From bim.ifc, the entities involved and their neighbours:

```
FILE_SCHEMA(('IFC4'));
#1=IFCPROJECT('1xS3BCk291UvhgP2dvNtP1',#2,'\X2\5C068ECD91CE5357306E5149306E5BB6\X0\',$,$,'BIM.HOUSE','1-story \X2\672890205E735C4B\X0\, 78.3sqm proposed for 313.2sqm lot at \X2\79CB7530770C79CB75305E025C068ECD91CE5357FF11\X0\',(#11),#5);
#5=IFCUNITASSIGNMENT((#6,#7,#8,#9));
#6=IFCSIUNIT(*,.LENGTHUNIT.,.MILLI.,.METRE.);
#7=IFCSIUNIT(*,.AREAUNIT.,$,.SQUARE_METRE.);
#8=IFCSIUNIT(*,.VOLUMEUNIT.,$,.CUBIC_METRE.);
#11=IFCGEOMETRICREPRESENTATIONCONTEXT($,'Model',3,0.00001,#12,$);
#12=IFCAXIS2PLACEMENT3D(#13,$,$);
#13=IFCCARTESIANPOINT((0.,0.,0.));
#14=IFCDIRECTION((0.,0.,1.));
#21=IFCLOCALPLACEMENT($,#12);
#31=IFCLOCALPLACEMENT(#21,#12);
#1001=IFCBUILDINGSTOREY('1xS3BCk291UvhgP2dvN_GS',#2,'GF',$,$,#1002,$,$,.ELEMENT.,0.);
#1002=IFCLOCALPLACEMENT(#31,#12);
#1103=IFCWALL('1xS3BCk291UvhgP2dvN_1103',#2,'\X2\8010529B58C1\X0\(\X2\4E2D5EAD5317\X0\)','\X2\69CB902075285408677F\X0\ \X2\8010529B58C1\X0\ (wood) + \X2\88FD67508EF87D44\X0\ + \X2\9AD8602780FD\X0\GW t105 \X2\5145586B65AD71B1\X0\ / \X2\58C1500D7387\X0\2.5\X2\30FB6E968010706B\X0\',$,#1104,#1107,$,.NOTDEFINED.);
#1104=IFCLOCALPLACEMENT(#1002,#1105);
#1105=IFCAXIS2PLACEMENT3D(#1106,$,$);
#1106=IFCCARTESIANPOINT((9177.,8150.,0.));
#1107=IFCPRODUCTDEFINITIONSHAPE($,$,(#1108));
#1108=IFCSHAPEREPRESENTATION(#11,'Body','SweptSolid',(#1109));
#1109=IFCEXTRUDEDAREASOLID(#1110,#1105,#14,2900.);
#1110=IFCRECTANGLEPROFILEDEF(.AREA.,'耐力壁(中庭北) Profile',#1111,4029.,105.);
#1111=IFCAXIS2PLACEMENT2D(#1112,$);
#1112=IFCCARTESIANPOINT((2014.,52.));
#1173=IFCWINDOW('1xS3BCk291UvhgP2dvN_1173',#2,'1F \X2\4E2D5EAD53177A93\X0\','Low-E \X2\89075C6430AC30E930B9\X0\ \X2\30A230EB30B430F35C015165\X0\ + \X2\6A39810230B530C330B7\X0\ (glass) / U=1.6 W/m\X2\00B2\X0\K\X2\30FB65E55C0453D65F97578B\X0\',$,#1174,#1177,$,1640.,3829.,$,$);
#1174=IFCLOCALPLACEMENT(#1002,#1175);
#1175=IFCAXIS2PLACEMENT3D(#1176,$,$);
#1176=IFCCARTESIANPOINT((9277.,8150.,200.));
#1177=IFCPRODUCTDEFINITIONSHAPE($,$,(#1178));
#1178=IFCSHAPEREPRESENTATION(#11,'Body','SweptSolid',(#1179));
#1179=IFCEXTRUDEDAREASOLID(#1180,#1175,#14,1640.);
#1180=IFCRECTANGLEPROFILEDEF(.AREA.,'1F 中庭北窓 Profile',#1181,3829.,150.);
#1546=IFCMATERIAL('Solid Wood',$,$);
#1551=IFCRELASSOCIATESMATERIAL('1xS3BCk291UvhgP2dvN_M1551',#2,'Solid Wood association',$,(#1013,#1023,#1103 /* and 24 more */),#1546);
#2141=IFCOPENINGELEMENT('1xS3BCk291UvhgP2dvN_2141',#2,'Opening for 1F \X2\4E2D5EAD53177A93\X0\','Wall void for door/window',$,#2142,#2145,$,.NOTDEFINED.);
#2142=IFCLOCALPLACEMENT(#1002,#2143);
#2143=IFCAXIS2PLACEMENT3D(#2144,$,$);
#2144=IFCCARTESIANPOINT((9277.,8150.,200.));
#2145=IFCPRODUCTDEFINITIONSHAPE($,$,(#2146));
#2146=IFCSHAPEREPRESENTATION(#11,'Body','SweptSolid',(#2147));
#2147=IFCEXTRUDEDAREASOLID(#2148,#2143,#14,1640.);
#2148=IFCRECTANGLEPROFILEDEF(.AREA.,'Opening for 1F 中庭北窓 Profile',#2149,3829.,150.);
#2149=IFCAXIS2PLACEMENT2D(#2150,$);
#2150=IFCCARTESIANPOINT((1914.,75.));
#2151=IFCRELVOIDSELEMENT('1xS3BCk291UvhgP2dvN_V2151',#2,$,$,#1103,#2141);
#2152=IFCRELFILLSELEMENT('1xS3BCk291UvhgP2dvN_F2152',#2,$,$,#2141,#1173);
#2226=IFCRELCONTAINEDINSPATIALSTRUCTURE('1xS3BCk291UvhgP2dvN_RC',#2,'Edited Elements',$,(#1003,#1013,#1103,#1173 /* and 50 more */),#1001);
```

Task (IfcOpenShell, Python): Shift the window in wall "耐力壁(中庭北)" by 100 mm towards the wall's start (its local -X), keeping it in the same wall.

```python
import ifcopenshell
import ifcopenshell.api.geometry
import ifcopenshell.util.placement
import ifcopenshell.util.unit

model = ifcopenshell.open("bim.ifc")
unit_scale = ifcopenshell.util.unit.calculate_unit_scale(model)

window = model.by_id(1173)
opening = window.FillsVoids[0].RelatingOpeningElement
wall = opening.VoidsElements[0].RelatingBuildingElement

wall_matrix = ifcopenshell.util.placement.get_local_placement(wall.ObjectPlacement)
shift = wall_matrix[:3, 0] * -0.1 / unit_scale
before = ifcopenshell.util.placement.get_local_placement(window.ObjectPlacement)[:3, 3].copy()

# The window is not placed relative to its opening, so move both.
for product in (opening, window):
    matrix = ifcopenshell.util.placement.get_local_placement(product.ObjectPlacement)
    matrix[:3, 3] += shift
    ifcopenshell.api.geometry.edit_object_placement(model, product=product, matrix=matrix, is_si=False)

after = ifcopenshell.util.placement.get_local_placement(window.ObjectPlacement)[:3, 3]
print("window moved by", (after - before).round(3) + 0.0)

model.write("bim-out.ifc")
```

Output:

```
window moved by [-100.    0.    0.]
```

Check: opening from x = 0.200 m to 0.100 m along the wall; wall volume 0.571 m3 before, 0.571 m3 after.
